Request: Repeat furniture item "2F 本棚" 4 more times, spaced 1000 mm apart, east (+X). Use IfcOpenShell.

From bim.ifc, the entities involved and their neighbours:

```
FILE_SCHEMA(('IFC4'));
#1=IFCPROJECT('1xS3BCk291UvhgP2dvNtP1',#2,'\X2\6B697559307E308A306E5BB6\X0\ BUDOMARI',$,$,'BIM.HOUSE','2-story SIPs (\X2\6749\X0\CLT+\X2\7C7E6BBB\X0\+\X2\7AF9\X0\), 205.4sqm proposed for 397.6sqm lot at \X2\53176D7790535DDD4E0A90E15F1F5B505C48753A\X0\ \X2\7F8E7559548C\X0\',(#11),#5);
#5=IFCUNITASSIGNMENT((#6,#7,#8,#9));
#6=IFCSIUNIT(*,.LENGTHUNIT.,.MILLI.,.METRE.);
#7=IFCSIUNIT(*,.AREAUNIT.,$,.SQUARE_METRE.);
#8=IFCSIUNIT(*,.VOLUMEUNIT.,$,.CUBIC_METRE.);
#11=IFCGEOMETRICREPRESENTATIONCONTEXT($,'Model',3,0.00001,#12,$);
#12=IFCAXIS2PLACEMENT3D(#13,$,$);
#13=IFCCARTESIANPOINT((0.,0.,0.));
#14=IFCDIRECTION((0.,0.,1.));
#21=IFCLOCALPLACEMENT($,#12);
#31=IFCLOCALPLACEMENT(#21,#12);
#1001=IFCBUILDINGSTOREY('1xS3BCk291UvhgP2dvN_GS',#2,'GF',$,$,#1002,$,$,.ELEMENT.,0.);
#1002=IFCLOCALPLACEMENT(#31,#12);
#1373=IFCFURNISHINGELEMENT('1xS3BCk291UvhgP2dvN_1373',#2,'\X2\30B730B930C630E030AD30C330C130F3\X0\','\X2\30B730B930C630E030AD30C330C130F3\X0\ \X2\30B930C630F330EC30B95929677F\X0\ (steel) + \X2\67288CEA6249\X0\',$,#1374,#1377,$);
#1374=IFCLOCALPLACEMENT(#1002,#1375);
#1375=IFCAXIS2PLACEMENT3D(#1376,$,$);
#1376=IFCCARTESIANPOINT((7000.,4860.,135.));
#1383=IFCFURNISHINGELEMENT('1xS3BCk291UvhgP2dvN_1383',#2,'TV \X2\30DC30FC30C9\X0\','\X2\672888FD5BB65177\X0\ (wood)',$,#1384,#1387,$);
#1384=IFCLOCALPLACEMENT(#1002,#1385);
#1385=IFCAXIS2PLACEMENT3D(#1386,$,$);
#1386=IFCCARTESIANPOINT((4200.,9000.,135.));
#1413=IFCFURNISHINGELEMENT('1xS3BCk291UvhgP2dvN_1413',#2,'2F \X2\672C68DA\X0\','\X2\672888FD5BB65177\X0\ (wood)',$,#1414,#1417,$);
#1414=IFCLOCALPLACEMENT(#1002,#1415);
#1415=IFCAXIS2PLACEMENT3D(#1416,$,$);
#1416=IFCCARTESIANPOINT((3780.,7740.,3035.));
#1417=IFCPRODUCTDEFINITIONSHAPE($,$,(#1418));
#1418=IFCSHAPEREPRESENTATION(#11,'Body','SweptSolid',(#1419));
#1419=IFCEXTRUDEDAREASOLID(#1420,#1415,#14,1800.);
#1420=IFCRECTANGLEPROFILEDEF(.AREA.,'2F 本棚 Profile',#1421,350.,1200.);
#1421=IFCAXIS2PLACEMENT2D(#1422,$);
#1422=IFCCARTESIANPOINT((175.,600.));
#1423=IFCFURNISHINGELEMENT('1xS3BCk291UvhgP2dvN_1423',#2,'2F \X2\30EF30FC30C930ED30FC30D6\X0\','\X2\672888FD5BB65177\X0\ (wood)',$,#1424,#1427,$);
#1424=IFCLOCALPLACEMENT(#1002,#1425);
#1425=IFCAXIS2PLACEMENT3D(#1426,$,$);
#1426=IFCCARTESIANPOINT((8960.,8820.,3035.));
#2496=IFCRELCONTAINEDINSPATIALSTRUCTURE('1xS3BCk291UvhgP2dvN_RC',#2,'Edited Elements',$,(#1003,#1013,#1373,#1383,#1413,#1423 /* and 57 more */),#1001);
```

```python
import numpy as np
import ifcopenshell
import ifcopenshell.api.geometry
import ifcopenshell.api.root
import ifcopenshell.util.element
import ifcopenshell.util.placement
import ifcopenshell.util.unit

model = ifcopenshell.open("bim.ifc")
unit_scale = ifcopenshell.util.unit.calculate_unit_scale(model)


def reuse_history(source, copy):
    """copy_class also copies each property set's owner history, people and application; keep the originals."""
    for rel in copy.IsDefinedBy:
        if rel.is_a("IfcRelDefinesByProperties") and (history := rel.RelatingPropertyDefinition.OwnerHistory):
            rel.RelatingPropertyDefinition.OwnerHistory = source.OwnerHistory
            ifcopenshell.util.element.remove_deep2(model, history)


source = model.by_id(1413)
base = ifcopenshell.util.placement.get_local_placement(source.ObjectPlacement)
step = np.array([1.0, 0.0, 0.0]) * 1 / unit_scale

for i in range(1, 5):
    copy = ifcopenshell.api.root.copy_class(model, product=source)
    copy.Representation = ifcopenshell.util.element.copy_deep(
        model, source.Representation, exclude=["IfcGeometricRepresentationContext", "IfcRepresentationMap"]
    )
    reuse_history(source, copy)
    matrix = base.copy()
    matrix[:3, 3] += i * step
    print("added at", matrix[:3, 3].round(3) + 0.0)
    ifcopenshell.api.geometry.edit_object_placement(model, product=copy, matrix=matrix, is_si=False)

model.write("bim_v2.ifc")
```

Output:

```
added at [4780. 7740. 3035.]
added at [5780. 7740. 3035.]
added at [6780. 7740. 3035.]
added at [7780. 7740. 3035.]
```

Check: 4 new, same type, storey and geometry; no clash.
